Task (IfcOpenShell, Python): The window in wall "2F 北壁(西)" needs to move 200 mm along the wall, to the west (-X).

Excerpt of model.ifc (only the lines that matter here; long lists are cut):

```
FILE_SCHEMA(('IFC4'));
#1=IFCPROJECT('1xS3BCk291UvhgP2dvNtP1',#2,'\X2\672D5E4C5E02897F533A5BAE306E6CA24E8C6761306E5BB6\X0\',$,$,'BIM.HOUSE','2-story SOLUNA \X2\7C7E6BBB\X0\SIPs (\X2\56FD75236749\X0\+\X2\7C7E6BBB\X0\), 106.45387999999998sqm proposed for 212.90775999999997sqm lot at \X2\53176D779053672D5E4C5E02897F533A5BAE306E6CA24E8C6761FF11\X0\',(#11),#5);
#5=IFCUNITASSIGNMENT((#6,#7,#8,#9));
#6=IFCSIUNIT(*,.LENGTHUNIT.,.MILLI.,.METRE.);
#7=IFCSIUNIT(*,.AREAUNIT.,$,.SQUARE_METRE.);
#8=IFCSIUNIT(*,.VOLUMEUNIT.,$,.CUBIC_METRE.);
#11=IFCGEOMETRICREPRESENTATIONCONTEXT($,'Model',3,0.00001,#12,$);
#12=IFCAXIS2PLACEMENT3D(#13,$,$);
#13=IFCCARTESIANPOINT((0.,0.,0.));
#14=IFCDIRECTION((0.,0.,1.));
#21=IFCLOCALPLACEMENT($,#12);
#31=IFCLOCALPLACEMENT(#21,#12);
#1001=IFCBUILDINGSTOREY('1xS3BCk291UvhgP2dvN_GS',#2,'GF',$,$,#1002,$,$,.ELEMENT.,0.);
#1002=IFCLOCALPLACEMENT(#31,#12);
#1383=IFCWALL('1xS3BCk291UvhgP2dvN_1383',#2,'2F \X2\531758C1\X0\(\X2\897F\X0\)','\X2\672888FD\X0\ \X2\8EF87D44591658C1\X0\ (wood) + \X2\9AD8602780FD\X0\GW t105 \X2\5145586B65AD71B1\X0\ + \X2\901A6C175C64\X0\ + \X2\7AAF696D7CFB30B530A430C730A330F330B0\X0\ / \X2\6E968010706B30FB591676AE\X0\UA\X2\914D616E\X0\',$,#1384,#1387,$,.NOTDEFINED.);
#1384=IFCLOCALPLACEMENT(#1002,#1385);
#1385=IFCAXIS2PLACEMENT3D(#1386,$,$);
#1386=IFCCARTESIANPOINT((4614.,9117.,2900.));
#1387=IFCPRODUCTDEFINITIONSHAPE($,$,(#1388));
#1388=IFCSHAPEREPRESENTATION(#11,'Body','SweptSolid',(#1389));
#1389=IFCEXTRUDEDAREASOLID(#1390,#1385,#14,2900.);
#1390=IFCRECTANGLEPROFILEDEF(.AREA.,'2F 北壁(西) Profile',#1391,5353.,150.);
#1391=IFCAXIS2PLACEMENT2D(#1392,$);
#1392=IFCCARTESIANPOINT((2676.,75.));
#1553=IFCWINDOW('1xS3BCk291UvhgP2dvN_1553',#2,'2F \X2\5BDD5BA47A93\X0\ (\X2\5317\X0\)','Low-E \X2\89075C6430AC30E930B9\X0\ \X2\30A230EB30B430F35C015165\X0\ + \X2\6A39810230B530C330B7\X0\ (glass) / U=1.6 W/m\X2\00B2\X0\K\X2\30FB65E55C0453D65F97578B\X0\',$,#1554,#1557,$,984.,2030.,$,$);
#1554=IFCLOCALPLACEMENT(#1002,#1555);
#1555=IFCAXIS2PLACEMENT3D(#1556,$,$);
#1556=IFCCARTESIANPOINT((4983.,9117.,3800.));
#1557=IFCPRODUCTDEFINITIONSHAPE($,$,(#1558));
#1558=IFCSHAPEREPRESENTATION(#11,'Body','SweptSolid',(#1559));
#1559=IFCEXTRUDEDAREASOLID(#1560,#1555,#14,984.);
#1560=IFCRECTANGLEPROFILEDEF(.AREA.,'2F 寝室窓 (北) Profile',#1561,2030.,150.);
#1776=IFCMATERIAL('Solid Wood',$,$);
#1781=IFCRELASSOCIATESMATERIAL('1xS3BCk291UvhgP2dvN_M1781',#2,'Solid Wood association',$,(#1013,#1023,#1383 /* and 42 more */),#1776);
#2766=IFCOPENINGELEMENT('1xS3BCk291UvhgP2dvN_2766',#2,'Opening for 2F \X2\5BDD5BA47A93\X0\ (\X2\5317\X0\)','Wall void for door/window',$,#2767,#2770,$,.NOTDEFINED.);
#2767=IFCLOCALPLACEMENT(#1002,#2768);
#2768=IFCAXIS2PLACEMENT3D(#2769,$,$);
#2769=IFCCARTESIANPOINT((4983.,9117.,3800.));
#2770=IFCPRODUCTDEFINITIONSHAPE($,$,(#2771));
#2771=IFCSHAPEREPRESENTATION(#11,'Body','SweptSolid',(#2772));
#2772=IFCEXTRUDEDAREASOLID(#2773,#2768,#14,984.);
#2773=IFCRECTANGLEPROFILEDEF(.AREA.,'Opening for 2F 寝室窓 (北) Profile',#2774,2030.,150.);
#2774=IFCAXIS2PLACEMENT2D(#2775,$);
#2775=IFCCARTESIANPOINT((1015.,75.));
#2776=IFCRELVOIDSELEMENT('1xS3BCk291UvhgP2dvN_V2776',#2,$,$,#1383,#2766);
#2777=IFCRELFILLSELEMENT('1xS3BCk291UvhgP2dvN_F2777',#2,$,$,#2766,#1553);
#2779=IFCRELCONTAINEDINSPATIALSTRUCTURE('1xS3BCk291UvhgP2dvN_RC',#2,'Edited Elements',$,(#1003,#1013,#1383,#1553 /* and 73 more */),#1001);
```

```python
import ifcopenshell
import ifcopenshell.api.geometry
import ifcopenshell.util.placement
import ifcopenshell.util.unit

model = ifcopenshell.open("model.ifc")
unit_scale = ifcopenshell.util.unit.calculate_unit_scale(model)

window = model.by_guid("1xS3BCk291UvhgP2dvN_1553")
opening = window.FillsVoids[0].RelatingOpeningElement
wall = opening.VoidsElements[0].RelatingBuildingElement

wall_matrix = ifcopenshell.util.placement.get_local_placement(wall.ObjectPlacement)
shift = wall_matrix[:3, 0] * -0.2 / unit_scale
before = ifcopenshell.util.placement.get_local_placement(window.ObjectPlacement)[:3, 3].copy()

# The window is not placed relative to its opening, so move both.
for product in (opening, window):
    matrix = ifcopenshell.util.placement.get_local_placement(product.ObjectPlacement)
    matrix[:3, 3] += shift
    ifcopenshell.api.geometry.edit_object_placement(model, product=product, matrix=matrix, is_si=False)

after = ifcopenshell.util.placement.get_local_placement(window.ObjectPlacement)[:3, 3]
print("window moved by", (after - before).round(3) + 0.0)

model.write("model_updated.ifc")
```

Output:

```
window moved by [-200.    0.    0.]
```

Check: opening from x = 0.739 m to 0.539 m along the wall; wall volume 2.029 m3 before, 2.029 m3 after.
